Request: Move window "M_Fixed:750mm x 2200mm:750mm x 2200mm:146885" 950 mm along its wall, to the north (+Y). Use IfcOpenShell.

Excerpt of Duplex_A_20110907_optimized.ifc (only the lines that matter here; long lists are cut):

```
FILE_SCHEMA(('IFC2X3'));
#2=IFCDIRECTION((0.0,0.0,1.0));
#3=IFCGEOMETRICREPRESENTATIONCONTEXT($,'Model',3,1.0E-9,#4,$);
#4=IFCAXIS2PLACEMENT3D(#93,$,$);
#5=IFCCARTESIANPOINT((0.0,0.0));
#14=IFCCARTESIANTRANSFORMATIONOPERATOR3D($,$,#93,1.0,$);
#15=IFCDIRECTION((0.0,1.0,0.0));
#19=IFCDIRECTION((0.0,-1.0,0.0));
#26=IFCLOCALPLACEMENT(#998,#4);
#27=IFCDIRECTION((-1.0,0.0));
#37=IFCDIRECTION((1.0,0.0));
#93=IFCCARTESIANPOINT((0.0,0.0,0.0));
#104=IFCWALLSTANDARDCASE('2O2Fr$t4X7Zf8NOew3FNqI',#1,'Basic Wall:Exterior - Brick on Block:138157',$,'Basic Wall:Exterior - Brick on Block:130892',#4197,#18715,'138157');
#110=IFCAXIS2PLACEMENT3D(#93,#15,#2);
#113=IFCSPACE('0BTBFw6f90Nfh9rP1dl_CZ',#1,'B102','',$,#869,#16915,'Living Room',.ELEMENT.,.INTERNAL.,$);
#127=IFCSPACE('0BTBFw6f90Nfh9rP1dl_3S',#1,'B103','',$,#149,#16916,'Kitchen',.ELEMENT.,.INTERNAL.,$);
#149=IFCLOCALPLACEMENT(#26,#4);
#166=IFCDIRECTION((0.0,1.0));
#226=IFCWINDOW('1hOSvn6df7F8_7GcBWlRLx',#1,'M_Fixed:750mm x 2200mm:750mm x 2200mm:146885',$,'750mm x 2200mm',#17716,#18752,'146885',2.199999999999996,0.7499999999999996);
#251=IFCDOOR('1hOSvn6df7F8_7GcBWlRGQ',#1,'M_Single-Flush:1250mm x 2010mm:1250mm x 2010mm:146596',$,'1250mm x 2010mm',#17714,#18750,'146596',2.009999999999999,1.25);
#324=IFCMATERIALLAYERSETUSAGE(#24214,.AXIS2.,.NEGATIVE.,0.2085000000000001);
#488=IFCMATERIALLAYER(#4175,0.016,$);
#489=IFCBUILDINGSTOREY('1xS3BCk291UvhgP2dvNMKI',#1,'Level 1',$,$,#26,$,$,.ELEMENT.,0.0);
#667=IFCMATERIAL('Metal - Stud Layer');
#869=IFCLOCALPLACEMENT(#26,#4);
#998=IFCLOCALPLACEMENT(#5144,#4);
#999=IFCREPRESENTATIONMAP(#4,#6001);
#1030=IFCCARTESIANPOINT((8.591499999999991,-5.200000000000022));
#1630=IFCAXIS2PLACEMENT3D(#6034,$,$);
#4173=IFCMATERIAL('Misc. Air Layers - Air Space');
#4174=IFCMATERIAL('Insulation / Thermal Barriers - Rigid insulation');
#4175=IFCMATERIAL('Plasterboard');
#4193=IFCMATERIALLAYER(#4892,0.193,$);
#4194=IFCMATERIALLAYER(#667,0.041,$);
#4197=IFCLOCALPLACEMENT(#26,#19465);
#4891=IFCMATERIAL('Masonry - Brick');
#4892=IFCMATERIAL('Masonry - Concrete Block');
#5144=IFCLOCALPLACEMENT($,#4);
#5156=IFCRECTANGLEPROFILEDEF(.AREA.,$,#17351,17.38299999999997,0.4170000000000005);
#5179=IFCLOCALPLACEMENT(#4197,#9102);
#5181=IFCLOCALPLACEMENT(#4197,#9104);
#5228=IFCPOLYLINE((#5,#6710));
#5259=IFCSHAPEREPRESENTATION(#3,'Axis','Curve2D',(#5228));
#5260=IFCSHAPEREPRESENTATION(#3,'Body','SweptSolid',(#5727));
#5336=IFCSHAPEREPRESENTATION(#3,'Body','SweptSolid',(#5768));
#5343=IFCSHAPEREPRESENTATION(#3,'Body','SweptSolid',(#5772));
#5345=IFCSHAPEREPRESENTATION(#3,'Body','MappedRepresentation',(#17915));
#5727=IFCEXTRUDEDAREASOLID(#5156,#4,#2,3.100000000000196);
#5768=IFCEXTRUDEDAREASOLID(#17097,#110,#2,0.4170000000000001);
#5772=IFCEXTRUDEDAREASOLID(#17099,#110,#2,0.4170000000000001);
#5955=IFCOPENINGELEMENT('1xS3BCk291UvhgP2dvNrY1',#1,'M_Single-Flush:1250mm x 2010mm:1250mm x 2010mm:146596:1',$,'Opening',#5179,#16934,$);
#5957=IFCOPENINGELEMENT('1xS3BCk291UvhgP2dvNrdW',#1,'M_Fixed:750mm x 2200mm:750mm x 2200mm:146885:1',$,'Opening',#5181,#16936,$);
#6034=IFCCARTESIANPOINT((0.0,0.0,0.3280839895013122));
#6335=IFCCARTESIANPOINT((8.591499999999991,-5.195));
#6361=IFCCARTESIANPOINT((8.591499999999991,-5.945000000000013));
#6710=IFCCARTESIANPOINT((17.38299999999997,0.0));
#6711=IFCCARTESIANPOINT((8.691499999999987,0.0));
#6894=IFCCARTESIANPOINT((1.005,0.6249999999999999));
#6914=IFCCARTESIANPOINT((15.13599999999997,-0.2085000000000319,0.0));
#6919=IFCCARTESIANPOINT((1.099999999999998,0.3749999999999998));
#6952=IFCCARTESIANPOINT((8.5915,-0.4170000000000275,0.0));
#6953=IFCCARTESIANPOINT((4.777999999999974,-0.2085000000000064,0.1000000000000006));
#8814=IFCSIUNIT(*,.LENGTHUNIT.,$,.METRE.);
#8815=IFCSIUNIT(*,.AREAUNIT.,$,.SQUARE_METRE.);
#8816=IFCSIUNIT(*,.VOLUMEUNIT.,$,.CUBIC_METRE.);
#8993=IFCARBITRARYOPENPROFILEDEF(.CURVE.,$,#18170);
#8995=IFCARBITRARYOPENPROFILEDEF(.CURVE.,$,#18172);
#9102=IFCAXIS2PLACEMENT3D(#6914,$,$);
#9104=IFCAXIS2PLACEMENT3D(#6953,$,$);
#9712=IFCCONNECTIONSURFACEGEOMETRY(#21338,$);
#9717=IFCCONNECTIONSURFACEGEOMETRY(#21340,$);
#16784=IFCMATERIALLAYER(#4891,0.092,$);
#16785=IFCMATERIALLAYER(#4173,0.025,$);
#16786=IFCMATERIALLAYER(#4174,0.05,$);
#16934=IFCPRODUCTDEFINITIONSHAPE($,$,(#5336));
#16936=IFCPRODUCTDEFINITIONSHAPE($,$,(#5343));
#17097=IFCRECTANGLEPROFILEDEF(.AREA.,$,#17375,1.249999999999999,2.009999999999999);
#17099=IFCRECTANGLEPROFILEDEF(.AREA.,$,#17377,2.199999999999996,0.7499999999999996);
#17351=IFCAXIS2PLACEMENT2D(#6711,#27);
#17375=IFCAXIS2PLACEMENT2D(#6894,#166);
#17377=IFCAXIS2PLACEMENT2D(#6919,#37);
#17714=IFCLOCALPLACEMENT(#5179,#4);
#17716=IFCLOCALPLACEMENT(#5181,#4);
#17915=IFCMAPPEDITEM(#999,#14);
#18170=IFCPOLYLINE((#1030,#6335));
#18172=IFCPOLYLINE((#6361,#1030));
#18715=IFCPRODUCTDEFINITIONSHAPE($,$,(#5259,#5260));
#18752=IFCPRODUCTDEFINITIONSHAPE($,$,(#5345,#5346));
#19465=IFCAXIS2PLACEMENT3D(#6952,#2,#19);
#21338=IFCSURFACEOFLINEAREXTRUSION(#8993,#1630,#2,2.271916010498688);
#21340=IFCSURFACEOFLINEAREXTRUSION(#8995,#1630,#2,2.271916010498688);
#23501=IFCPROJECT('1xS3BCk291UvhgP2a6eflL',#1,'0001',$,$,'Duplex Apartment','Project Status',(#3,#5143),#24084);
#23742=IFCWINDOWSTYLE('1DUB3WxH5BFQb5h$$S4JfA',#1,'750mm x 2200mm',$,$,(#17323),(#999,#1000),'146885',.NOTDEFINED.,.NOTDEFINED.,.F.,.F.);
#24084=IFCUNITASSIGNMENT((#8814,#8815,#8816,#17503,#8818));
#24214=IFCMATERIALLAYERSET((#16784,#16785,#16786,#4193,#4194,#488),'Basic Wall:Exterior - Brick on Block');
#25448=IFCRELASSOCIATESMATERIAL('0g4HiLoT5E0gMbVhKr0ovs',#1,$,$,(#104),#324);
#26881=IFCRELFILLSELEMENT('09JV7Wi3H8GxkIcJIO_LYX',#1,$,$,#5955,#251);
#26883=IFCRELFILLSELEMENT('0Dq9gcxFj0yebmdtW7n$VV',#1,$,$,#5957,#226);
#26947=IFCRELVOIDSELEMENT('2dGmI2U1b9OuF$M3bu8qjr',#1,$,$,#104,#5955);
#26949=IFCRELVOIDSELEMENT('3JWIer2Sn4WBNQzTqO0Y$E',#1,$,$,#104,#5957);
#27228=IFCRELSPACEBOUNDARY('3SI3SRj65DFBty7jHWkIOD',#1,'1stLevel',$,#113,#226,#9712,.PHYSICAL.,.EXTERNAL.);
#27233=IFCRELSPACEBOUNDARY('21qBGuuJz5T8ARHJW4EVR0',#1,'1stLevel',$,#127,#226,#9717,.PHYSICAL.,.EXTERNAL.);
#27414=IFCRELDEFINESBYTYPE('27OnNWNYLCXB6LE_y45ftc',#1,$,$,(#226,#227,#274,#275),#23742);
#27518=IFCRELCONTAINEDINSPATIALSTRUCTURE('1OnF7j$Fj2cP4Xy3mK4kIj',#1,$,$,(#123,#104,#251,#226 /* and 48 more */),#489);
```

```python
import numpy as np
import ifcopenshell
import ifcopenshell.api.geometry
import ifcopenshell.util.placement
import ifcopenshell.util.unit

model = ifcopenshell.open("Duplex_A_20110907_optimized.ifc")
unit_scale = ifcopenshell.util.unit.calculate_unit_scale(model)

window = model.by_id(226)
opening = window.FillsVoids[0].RelatingOpeningElement
wall = opening.VoidsElements[0].RelatingBuildingElement

wall_matrix = ifcopenshell.util.placement.get_local_placement(wall.ObjectPlacement)
shift = wall_matrix[:3, 0] * -0.95 / unit_scale
before = ifcopenshell.util.placement.get_local_placement(window.ObjectPlacement)[:3, 3].copy()

# The window is placed relative to its opening, so it follows when the opening moves.
matrix = ifcopenshell.util.placement.get_local_placement(opening.ObjectPlacement)
matrix[:3, 3] += shift
ifcopenshell.api.geometry.edit_object_placement(
    model, product=opening, matrix=matrix, is_si=False, should_transform_children=True
)

# Space boundary surfaces are stored in each space's coordinates; move them too.
for rel in window.ProvidesBoundaries:
    if not rel.ConnectionGeometry:
        continue
    surface = rel.ConnectionGeometry.SurfaceOnRelatingElement
    space_matrix = ifcopenshell.util.placement.get_local_placement(rel.RelatingSpace.ObjectPlacement)
    point = np.array(surface.Position.Location.Coordinates) + space_matrix[:3, :3].T @ shift
    surface.Position = model.createIfcAxis2Placement3D(
        model.createIfcCartesianPoint(point.tolist()), surface.Position.Axis, surface.Position.RefDirection
    )

after = ifcopenshell.util.placement.get_local_placement(window.ObjectPlacement)[:3, 3]
print("window moved by", (after - before).round(3) + 0.0)

model.write("Duplex_A_20110907_optimized_edited.ifc")
```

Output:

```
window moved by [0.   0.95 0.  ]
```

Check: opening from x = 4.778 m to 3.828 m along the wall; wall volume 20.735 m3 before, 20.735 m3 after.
